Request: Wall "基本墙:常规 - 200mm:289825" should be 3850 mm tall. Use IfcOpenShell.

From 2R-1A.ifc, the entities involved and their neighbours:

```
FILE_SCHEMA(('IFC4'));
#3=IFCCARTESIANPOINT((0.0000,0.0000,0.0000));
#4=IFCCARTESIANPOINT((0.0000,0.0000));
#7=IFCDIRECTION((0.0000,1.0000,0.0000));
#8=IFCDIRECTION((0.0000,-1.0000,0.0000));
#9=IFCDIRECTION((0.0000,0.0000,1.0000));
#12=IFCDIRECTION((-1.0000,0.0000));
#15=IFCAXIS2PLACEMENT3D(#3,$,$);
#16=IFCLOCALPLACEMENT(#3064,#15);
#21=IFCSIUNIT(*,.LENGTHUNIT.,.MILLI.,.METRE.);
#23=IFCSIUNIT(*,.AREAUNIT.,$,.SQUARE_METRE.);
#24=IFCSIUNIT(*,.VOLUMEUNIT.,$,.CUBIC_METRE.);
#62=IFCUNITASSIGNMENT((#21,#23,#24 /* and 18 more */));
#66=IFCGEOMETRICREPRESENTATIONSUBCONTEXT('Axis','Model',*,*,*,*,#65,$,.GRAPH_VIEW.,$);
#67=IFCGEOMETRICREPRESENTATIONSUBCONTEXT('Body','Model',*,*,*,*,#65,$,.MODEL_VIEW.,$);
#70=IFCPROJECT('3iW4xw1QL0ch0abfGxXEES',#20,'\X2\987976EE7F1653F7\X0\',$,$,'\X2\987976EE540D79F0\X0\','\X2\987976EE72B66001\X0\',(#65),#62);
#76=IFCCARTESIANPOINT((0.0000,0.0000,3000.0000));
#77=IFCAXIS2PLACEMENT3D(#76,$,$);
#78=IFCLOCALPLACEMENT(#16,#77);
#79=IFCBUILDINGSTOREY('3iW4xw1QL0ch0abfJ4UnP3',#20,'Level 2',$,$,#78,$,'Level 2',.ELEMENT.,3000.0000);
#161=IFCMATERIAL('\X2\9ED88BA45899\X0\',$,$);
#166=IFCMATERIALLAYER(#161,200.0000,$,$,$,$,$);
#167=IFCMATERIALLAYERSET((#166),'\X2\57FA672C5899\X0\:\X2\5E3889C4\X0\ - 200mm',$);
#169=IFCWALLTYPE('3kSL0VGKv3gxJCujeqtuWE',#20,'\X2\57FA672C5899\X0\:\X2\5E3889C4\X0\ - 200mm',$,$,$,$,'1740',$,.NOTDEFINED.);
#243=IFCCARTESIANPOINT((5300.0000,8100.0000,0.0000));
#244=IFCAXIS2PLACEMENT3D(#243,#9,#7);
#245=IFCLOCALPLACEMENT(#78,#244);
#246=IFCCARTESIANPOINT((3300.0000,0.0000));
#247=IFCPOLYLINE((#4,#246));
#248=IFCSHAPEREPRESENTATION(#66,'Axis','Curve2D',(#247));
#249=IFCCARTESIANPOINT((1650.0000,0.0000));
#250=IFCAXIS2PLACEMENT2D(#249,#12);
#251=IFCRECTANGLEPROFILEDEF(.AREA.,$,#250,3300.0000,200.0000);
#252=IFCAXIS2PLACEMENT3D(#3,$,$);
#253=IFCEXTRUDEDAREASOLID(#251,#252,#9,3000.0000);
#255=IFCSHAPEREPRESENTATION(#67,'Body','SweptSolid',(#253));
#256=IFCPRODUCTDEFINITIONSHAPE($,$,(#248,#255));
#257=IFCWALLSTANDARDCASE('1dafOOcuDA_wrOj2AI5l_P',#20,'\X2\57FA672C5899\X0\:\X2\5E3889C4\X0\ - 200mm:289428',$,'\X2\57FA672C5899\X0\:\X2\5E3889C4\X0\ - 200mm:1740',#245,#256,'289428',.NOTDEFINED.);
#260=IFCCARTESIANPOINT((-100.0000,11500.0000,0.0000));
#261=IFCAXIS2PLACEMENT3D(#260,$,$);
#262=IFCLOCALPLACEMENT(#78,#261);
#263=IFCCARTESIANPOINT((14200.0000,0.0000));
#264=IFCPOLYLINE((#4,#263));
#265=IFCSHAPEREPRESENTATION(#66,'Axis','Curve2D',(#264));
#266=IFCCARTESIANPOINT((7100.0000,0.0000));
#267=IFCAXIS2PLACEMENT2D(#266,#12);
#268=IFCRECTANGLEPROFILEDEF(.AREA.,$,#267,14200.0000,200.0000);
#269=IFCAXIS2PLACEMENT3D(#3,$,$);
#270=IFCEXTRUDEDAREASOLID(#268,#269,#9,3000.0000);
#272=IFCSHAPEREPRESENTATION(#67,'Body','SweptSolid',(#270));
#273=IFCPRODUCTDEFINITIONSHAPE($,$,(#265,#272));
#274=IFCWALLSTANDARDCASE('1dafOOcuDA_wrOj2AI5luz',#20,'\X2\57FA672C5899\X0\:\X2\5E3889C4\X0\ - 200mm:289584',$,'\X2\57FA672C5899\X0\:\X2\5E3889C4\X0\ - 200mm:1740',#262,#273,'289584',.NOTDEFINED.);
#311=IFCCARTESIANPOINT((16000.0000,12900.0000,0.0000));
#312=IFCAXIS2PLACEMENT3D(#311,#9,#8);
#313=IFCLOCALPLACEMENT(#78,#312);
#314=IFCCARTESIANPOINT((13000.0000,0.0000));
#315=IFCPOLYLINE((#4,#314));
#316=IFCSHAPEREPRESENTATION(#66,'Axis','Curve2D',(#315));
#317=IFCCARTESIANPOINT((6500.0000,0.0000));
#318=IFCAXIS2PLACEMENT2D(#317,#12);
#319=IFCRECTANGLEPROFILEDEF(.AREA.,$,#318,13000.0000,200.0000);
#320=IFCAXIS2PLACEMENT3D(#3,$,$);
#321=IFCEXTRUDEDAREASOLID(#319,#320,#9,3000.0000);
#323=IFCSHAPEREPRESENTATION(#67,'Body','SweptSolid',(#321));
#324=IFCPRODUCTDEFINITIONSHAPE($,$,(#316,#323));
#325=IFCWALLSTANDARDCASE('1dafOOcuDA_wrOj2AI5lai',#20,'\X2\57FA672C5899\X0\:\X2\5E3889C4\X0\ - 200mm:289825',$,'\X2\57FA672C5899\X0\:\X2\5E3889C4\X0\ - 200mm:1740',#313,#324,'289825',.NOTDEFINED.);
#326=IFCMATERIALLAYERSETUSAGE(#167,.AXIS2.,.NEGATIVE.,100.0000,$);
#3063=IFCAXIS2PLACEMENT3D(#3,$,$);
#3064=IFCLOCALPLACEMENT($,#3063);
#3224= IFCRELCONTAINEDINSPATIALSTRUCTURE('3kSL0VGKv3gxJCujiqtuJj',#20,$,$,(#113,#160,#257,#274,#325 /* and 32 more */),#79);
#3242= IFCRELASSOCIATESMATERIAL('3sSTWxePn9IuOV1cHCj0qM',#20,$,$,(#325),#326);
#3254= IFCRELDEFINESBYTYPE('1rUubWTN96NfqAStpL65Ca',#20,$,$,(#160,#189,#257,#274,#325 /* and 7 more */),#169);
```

```python
import ifcopenshell
import ifcopenshell.geom
import ifcopenshell.util.representation
import ifcopenshell.util.shape

model = ifcopenshell.open("2R-1A.ifc")
settings = ifcopenshell.geom.settings()


def volume(element):
    """Net volume in cubic metres, openings subtracted."""
    shape = ifcopenshell.geom.create_shape(settings, element)
    return ifcopenshell.util.shape.get_volume(shape.geometry)


wall = model.by_guid("1dafOOcuDA_wrOj2AI5lai")
before = volume(wall)

body = ifcopenshell.util.representation.get_representation(wall, "Model", "Body")
solid = body.Items[0]
old_height = solid.Depth
solid.Depth = 3850.0
after = volume(wall)

print(f"height {old_height:g} -> {solid.Depth:g}, volume {before:.3f} -> {after:.3f} m3")

model.write("2R-1A-out.ifc")
```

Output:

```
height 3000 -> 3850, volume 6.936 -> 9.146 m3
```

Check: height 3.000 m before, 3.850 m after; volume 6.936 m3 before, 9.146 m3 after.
